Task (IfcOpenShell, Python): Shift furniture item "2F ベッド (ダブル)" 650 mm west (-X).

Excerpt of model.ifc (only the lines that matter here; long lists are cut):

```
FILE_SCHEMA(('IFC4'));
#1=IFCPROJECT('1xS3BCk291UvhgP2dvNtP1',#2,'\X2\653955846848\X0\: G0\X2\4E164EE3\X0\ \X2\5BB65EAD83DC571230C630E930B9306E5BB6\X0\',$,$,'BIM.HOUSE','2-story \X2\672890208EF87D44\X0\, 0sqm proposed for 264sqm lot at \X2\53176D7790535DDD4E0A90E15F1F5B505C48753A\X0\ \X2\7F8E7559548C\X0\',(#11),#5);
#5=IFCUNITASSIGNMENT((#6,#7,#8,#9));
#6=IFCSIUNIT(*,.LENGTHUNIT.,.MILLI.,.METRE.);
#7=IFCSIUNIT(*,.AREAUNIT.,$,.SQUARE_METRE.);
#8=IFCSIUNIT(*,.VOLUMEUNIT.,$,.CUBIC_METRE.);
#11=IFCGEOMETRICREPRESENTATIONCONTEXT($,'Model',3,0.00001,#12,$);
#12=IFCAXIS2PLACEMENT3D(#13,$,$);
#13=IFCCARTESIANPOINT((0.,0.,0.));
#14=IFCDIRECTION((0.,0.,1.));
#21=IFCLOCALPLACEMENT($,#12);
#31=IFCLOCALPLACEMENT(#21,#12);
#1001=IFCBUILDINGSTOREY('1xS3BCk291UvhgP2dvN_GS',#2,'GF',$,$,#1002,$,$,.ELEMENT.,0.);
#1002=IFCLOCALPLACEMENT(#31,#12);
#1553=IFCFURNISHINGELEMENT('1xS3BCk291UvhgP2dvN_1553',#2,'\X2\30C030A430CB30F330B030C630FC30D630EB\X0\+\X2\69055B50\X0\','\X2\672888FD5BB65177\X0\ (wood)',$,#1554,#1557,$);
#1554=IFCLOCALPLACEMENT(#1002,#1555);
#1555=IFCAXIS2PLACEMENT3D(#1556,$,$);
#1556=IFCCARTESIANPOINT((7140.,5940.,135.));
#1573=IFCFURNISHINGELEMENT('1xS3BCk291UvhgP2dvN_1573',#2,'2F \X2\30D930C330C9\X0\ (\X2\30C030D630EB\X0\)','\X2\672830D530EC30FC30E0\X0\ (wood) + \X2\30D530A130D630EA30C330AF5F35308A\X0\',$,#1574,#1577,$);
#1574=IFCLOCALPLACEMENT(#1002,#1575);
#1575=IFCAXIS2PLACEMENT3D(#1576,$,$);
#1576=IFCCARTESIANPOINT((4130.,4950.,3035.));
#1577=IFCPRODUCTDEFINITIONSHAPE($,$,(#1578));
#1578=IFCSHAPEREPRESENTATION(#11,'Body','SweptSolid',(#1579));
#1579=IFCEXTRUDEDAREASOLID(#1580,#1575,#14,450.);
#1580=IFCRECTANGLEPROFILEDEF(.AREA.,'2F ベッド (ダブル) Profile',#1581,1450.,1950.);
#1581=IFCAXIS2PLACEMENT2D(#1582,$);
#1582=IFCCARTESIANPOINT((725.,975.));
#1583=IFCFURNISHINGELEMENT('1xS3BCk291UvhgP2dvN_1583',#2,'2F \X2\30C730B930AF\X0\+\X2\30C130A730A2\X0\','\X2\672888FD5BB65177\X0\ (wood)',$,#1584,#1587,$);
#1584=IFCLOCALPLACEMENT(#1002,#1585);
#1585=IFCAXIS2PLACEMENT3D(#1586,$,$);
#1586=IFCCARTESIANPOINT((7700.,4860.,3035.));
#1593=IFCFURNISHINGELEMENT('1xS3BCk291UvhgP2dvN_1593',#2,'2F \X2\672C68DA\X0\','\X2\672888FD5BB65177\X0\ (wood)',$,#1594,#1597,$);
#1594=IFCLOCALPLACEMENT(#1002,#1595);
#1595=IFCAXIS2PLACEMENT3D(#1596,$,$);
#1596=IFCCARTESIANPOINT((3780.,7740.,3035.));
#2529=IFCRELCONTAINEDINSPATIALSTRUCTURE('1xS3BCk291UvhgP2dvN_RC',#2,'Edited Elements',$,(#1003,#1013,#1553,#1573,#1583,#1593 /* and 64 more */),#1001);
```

```python
import ifcopenshell
import ifcopenshell.api.geometry
import ifcopenshell.util.placement
import ifcopenshell.util.unit

model = ifcopenshell.open("model.ifc")
unit_scale = ifcopenshell.util.unit.calculate_unit_scale(model)

item = model.by_guid("1xS3BCk291UvhgP2dvN_1573")
matrix = ifcopenshell.util.placement.get_local_placement(item.ObjectPlacement)
matrix[0, 3] -= 0.65 / unit_scale
ifcopenshell.api.geometry.edit_object_placement(model, product=item, matrix=matrix, is_si=False)

print(ifcopenshell.util.placement.get_local_placement(item.ObjectPlacement).round(3) + 0.0)

model.write("model-out.ifc")
```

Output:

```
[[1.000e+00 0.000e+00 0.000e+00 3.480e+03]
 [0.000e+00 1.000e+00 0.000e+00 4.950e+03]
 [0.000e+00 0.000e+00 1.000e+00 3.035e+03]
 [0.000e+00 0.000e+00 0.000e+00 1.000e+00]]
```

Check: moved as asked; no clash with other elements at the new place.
